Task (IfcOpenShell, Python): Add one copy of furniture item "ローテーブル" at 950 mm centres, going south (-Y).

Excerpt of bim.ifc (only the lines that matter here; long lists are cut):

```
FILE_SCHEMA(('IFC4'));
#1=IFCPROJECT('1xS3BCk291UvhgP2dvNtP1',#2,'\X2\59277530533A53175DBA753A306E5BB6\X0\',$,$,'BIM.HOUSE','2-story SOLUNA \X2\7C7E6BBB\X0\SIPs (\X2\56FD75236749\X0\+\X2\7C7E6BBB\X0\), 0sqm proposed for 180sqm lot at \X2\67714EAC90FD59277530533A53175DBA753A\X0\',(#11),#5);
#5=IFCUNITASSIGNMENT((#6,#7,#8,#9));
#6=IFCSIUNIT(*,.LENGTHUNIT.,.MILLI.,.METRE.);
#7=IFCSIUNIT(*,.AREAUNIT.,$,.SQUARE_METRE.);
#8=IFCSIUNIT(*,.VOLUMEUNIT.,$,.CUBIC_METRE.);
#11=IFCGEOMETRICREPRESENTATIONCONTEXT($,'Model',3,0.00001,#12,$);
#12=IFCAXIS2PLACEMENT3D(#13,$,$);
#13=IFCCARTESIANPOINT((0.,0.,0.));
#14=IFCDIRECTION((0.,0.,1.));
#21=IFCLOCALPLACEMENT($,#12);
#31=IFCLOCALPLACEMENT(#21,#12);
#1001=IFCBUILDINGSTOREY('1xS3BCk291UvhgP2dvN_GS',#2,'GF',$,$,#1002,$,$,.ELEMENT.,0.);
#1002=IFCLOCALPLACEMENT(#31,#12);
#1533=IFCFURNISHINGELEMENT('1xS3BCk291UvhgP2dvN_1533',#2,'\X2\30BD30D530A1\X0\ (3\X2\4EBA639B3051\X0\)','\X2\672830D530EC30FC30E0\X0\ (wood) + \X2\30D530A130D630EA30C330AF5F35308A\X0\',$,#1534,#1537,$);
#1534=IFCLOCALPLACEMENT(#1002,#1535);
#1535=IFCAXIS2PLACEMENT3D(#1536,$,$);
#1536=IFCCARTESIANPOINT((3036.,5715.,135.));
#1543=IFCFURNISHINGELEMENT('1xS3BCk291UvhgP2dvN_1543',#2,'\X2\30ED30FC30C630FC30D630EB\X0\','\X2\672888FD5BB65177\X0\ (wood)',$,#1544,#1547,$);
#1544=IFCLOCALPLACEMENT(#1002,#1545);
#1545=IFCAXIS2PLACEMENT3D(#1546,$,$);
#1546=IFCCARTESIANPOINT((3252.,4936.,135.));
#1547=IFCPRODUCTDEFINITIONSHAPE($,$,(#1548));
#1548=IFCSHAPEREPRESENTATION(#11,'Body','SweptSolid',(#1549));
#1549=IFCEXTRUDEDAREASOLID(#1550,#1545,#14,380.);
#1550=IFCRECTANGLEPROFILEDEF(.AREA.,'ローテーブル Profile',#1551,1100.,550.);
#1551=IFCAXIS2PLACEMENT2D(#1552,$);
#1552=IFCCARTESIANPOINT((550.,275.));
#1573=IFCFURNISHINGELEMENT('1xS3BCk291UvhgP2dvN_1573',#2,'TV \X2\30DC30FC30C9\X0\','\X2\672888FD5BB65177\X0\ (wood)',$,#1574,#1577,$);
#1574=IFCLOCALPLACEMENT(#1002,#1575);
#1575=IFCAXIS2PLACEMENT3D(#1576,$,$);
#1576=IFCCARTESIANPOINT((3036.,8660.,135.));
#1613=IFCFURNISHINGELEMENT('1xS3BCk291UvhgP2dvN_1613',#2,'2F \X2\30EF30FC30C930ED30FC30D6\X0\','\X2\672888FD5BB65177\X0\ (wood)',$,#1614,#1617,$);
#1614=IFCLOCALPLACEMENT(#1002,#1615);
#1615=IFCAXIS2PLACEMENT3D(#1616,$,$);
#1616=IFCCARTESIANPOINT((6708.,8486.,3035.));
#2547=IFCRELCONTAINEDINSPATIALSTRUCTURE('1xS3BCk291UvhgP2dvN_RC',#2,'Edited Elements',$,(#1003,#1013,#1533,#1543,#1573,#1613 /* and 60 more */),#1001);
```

```python
import numpy as np
import ifcopenshell
import ifcopenshell.api.geometry
import ifcopenshell.api.root
import ifcopenshell.util.element
import ifcopenshell.util.placement
import ifcopenshell.util.unit

model = ifcopenshell.open("bim.ifc")
unit_scale = ifcopenshell.util.unit.calculate_unit_scale(model)


def reuse_history(source, copy):
    """copy_class also copies each property set's owner history, people and application; keep the originals."""
    for rel in copy.IsDefinedBy:
        if rel.is_a("IfcRelDefinesByProperties") and (history := rel.RelatingPropertyDefinition.OwnerHistory):
            rel.RelatingPropertyDefinition.OwnerHistory = source.OwnerHistory
            ifcopenshell.util.element.remove_deep2(model, history)


source = model.by_guid("1xS3BCk291UvhgP2dvN_1543")
base = ifcopenshell.util.placement.get_local_placement(source.ObjectPlacement)
step = np.array([0.0, -1.0, 0.0]) * 0.95 / unit_scale

for i in range(1, 2):
    copy = ifcopenshell.api.root.copy_class(model, product=source)
    copy.Representation = ifcopenshell.util.element.copy_deep(
        model, source.Representation, exclude=["IfcGeometricRepresentationContext", "IfcRepresentationMap"]
    )
    reuse_history(source, copy)
    matrix = base.copy()
    matrix[:3, 3] += i * step
    print("added at", matrix[:3, 3].round(3) + 0.0)
    ifcopenshell.api.geometry.edit_object_placement(model, product=copy, matrix=matrix, is_si=False)

model.write("bim_updated.ifc")
```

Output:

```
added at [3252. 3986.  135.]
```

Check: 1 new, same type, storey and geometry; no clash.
